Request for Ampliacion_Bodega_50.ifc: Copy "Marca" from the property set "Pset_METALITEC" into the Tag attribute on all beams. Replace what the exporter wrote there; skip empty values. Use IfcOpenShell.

First a look at what the model holds.

```python
import ifcopenshell
import ifcopenshell.util.element

model = ifcopenshell.open("Ampliacion_Bodega_50.ifc")
print(model.schema)
beams = model.by_type("IfcBeam")
print(len(beams), "beams")
for e in beams[:8]:
    source = ifcopenshell.util.element.get_pset(e, "Pset_METALITEC", "Marca")
    target = e.Tag
    print(e.id(), repr(source), repr(target), sep=" | ")
```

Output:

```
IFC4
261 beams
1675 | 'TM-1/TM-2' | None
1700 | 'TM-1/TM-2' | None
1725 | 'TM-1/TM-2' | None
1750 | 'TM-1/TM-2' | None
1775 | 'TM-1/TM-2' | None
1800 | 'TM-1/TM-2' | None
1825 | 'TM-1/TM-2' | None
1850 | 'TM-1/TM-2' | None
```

```python
import ifcopenshell
import ifcopenshell.util.element

model = ifcopenshell.open("Ampliacion_Bodega_50.ifc")

count = 0
for e in model.by_type("IfcBeam"):
    value = ifcopenshell.util.element.get_pset(e, "Pset_METALITEC", "Marca")
    current = e.Tag
    if not value or not value.strip() or current == value:
        continue
    e.Tag = value
    count += 1

print(count, "beams updated")

model.write("Ampliacion_Bodega_50-out.ifc")
```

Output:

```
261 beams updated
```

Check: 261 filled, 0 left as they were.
